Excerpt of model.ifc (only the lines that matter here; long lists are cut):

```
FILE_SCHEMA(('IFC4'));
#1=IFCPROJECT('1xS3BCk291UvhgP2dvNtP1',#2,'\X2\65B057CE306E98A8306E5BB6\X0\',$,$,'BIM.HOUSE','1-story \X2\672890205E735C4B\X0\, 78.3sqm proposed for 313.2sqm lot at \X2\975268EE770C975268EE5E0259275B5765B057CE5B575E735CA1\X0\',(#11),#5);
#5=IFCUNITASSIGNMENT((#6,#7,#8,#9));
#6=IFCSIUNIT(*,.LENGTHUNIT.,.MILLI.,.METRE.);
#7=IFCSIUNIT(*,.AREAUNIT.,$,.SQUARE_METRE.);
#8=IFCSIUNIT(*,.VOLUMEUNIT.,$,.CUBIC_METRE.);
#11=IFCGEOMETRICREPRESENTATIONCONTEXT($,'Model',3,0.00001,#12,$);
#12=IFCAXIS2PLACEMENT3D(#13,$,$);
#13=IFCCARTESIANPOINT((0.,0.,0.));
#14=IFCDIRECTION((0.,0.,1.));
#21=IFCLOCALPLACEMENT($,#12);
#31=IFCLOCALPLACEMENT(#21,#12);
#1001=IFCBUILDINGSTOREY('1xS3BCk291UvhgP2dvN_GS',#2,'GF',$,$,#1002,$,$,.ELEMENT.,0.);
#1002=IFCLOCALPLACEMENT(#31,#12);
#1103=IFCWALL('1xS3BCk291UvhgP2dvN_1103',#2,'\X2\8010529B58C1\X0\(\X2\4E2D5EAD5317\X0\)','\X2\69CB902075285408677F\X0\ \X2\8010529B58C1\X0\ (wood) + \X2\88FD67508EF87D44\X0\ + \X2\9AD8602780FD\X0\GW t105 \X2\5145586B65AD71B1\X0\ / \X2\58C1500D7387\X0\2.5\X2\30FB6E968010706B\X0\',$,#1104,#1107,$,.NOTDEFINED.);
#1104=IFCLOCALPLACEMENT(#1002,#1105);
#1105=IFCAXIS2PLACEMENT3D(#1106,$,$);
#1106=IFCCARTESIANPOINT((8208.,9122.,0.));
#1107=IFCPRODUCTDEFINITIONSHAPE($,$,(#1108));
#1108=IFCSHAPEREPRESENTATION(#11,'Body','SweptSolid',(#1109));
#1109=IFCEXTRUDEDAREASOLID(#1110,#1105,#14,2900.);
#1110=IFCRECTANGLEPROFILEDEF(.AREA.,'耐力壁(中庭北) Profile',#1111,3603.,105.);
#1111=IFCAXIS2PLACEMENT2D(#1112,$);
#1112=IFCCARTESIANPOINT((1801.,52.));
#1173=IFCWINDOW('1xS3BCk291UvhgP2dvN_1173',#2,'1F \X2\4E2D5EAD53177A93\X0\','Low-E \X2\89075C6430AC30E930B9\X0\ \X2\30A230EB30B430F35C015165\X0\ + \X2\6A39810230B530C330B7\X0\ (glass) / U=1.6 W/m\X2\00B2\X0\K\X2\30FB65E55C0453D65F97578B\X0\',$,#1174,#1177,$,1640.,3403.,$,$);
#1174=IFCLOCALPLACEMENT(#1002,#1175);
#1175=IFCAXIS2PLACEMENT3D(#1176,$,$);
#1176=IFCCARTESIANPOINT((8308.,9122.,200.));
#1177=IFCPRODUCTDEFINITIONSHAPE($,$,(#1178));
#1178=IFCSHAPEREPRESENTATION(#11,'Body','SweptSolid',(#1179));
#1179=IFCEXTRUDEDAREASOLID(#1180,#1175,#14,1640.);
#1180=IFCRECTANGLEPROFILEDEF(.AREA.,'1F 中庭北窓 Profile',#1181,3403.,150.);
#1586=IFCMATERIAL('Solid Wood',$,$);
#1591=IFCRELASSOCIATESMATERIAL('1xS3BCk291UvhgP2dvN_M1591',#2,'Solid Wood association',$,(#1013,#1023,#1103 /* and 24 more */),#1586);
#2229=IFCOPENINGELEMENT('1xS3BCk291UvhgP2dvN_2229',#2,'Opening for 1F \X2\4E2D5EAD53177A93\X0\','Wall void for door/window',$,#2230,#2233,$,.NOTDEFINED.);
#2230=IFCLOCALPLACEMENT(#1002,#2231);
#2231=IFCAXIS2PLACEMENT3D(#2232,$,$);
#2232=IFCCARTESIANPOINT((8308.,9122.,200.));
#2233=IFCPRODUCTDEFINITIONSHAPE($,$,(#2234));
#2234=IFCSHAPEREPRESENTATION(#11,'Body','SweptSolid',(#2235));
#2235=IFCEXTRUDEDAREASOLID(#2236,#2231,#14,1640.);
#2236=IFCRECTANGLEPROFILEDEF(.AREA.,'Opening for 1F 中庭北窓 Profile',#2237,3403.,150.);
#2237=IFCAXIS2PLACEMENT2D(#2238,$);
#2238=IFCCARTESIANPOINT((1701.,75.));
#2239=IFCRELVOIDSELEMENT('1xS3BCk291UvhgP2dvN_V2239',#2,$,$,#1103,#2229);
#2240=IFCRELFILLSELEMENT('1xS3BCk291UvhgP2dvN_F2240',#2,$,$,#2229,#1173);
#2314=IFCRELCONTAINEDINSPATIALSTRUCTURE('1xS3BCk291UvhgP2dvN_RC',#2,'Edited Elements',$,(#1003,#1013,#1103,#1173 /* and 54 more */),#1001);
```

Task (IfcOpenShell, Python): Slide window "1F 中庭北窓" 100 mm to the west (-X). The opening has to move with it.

```python
import ifcopenshell
import ifcopenshell.api.geometry
import ifcopenshell.util.placement
import ifcopenshell.util.unit

model = ifcopenshell.open("model.ifc")
unit_scale = ifcopenshell.util.unit.calculate_unit_scale(model)

window = model.by_guid("1xS3BCk291UvhgP2dvN_1173")
opening = window.FillsVoids[0].RelatingOpeningElement
wall = opening.VoidsElements[0].RelatingBuildingElement

wall_matrix = ifcopenshell.util.placement.get_local_placement(wall.ObjectPlacement)
shift = wall_matrix[:3, 0] * -0.1 / unit_scale
before = ifcopenshell.util.placement.get_local_placement(window.ObjectPlacement)[:3, 3].copy()

# The window is not placed relative to its opening, so move both.
for product in (opening, window):
    matrix = ifcopenshell.util.placement.get_local_placement(product.ObjectPlacement)
    matrix[:3, 3] += shift
    ifcopenshell.api.geometry.edit_object_placement(model, product=product, matrix=matrix, is_si=False)

after = ifcopenshell.util.placement.get_local_placement(window.ObjectPlacement)[:3, 3]
print("window moved by", (after - before).round(3) + 0.0)

model.write("model_v2.ifc")
```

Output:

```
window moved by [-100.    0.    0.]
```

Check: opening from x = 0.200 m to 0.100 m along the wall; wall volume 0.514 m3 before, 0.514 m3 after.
